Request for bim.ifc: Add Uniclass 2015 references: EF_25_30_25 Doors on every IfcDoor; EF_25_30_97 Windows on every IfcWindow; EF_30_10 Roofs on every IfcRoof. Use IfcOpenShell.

First a look at what the model holds.

```python
import ifcopenshell

model = ifcopenshell.open("bim.ifc")
print(model.schema)
print("classifications:", [c.Name for c in model.by_type("IfcClassification")])
for ifc_class in ("IfcDoor", "IfcRoof", "IfcStair", "IfcWall", "IfcWindow"):
    print(ifc_class, len(model.by_type(ifc_class)))
```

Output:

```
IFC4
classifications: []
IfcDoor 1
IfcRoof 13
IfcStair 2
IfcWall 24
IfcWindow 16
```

```python
import ifcopenshell
import ifcopenshell.api.classification

model = ifcopenshell.open("bim.ifc")

system = ifcopenshell.api.classification.add_classification(model, classification="Uniclass 2015")

codes = {
    "IfcDoor": ("EF_25_30_25", "Doors"),
    "IfcWindow": ("EF_25_30_97", "Windows"),
    "IfcRoof": ("EF_30_10", "Roofs"),
}
for ifc_class, (code, name) in codes.items():
    products = model.by_type(ifc_class)
    ifcopenshell.api.classification.add_reference(
        model, products=products, classification=system, identification=code, name=name
    )
    print(code, len(products))

model.write("bim_edited.ifc")
```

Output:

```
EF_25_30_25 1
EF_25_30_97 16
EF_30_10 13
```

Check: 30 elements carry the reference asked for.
